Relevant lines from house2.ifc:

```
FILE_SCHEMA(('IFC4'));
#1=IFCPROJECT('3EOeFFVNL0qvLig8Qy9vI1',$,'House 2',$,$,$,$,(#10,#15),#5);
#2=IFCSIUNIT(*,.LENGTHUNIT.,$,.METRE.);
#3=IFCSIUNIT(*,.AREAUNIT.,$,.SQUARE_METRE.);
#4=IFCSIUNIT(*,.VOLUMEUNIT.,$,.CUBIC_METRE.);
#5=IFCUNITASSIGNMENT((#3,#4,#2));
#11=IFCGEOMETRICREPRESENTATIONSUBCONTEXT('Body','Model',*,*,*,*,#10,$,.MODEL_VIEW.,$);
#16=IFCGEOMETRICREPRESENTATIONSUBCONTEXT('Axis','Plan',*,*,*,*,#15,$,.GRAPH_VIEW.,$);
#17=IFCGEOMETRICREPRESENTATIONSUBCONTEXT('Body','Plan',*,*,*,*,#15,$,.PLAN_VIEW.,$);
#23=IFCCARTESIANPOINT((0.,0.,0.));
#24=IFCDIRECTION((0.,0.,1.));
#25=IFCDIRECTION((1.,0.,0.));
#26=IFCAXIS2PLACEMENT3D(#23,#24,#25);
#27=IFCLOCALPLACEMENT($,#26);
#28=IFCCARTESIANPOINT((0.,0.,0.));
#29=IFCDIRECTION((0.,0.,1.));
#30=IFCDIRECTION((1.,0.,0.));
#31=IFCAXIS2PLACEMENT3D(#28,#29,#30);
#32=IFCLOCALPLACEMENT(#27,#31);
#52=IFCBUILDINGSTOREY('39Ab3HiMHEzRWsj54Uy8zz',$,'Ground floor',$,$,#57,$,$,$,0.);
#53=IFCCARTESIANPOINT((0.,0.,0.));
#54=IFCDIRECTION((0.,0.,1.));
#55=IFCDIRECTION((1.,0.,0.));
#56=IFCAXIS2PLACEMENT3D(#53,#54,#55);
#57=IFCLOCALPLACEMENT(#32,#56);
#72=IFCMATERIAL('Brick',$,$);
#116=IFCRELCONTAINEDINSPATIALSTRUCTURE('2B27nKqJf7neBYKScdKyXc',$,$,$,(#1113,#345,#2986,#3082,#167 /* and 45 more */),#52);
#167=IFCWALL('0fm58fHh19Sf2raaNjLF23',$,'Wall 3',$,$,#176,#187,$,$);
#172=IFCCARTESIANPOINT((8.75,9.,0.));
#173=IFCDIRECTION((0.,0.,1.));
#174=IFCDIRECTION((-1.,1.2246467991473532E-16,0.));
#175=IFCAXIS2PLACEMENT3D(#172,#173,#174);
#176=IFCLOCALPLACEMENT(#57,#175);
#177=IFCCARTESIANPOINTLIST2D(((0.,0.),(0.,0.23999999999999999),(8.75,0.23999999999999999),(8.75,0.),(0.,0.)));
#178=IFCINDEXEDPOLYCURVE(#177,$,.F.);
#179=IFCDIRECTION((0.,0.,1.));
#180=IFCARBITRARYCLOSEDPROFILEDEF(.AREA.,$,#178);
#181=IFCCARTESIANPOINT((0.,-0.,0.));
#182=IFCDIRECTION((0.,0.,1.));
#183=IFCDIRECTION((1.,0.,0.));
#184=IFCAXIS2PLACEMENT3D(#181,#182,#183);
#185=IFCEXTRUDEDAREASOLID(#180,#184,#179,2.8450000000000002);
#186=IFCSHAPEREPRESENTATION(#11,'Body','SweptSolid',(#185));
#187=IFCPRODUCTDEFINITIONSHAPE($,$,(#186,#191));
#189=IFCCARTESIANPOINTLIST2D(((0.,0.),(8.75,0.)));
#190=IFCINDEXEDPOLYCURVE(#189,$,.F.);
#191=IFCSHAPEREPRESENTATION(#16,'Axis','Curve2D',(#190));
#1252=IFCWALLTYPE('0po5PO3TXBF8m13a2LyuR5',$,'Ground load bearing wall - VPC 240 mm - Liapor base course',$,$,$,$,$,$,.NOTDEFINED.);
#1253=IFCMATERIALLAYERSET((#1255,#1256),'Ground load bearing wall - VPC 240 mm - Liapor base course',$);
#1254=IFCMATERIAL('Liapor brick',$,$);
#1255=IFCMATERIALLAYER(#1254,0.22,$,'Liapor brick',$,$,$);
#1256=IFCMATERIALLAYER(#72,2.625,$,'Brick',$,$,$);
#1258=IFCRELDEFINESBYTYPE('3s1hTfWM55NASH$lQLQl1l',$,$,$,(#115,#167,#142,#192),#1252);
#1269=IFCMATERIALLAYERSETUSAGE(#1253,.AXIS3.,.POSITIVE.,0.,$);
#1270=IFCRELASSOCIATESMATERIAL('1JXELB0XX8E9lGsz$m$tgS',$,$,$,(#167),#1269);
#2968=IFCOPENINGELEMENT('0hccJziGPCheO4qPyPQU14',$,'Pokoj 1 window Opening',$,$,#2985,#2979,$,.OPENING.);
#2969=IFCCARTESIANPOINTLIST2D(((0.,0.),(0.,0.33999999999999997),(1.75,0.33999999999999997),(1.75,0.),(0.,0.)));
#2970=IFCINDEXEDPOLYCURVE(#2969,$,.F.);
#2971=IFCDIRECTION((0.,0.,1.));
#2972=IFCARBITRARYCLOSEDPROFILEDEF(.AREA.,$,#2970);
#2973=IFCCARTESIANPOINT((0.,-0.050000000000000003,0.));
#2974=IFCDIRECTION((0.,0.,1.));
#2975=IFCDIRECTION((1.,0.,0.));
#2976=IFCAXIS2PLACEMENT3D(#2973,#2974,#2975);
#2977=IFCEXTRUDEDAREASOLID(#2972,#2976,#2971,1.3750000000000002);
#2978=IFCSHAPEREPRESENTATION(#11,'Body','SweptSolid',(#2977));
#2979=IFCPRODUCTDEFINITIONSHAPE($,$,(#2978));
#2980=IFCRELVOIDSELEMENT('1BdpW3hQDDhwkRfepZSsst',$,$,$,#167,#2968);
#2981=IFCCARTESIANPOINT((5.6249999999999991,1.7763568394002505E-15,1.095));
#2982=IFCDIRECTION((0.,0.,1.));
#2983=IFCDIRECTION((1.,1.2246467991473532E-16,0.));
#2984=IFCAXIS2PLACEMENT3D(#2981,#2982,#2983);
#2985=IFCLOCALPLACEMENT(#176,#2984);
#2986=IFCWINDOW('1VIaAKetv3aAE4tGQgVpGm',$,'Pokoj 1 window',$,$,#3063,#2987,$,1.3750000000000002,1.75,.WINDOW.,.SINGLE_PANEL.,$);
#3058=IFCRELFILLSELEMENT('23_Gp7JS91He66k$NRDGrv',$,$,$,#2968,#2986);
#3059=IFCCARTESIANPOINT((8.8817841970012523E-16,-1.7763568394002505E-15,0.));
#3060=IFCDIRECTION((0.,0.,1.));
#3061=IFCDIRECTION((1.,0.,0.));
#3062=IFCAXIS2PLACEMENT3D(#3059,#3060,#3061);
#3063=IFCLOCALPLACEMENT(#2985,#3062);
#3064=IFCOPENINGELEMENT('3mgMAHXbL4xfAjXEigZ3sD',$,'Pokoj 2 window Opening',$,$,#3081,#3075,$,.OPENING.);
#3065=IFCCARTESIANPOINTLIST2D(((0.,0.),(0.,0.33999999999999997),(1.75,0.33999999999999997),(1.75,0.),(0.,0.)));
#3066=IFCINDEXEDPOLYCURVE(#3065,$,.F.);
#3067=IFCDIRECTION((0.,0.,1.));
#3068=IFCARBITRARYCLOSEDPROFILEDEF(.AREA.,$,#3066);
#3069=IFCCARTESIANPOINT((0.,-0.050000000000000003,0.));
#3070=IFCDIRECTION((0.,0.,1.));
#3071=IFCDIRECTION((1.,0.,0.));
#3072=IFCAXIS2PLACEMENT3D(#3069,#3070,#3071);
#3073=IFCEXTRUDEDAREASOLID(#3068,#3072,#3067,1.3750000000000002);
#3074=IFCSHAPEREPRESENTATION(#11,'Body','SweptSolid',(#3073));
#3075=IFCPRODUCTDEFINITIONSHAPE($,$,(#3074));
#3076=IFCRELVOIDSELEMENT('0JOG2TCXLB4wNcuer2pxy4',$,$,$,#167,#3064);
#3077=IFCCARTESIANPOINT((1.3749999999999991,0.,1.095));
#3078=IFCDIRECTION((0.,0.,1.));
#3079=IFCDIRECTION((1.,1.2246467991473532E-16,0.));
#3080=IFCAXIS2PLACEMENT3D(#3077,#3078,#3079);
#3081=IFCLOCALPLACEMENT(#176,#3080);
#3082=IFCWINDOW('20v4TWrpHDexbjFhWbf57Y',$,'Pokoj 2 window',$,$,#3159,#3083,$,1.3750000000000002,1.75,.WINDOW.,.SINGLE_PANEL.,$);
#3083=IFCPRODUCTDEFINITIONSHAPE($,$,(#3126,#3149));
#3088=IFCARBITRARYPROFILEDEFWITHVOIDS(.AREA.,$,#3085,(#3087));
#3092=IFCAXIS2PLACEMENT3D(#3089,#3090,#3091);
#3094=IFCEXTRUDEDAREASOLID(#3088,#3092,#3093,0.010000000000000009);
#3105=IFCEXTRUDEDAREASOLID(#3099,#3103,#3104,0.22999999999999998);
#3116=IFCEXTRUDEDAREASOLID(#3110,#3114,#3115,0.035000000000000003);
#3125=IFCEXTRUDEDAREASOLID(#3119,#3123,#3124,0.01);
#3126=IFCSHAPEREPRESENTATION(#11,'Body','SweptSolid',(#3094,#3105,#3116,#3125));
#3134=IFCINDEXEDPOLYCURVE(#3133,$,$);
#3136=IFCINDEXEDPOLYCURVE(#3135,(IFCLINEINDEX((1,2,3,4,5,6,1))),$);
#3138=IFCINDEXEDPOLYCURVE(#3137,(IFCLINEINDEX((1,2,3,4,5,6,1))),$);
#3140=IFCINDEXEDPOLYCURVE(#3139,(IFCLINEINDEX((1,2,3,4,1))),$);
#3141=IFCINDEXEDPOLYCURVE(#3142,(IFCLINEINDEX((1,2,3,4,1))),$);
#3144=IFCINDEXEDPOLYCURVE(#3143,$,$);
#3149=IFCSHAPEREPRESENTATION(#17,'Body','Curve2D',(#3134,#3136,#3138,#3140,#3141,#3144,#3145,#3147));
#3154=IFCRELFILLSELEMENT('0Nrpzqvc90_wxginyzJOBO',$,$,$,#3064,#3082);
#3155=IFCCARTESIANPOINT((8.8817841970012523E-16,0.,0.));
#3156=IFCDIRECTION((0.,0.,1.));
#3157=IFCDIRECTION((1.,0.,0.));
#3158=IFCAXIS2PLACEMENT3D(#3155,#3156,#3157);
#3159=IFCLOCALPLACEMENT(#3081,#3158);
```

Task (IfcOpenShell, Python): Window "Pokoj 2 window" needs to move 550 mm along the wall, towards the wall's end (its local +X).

```python
import ifcopenshell
import ifcopenshell.api.geometry
import ifcopenshell.util.placement

model = ifcopenshell.open("house2.ifc")

window = model.by_id(3082)
opening = window.FillsVoids[0].RelatingOpeningElement
wall = opening.VoidsElements[0].RelatingBuildingElement

wall_matrix = ifcopenshell.util.placement.get_local_placement(wall.ObjectPlacement)
shift = wall_matrix[:3, 0] * 0.55
before = ifcopenshell.util.placement.get_local_placement(window.ObjectPlacement)[:3, 3].copy()

# The window is placed relative to its opening, so it follows when the opening moves.
matrix = ifcopenshell.util.placement.get_local_placement(opening.ObjectPlacement)
matrix[:3, 3] += shift
ifcopenshell.api.geometry.edit_object_placement(
    model, product=opening, matrix=matrix, is_si=False, should_transform_children=True
)

after = ifcopenshell.util.placement.get_local_placement(window.ObjectPlacement)[:3, 3]
print("window moved by", (after - before).round(3) + 0.0)

model.write("house2_v2.ifc")
```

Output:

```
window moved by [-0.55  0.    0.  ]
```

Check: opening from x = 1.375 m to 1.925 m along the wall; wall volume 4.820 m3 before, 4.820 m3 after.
